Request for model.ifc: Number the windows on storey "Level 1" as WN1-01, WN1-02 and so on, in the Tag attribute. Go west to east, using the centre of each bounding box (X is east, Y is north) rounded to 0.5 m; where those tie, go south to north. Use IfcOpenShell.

First a look at what the model holds.

```python
import ifcopenshell
import ifcopenshell.util.element
import ifcopenshell.util.placement

model = ifcopenshell.open("model.ifc")
print(model.schema)
storey = next(s for s in model.by_type("IfcBuildingStorey") if s.Name == "Level 1")
windows = [e for e in ifcopenshell.util.element.get_decomposition(storey) if e.is_a("IfcWindow")]
for e in sorted(windows, key=lambda e: e.id()):
    origin = ifcopenshell.util.placement.get_local_placement(e.ObjectPlacement)[:3, 3]
    print(e.id(), e.Tag, e.Name, origin.round(2) + 0.0, sep=" | ")
```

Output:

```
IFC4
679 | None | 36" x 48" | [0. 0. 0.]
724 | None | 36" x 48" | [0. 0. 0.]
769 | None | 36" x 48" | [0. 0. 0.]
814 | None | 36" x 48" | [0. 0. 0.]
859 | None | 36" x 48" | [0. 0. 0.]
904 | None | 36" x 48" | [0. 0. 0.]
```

```python
import ifcopenshell
import ifcopenshell.geom
import ifcopenshell.util.element
import ifcopenshell.util.shape

model = ifcopenshell.open("model.ifc")
settings = ifcopenshell.geom.settings()
settings.set("use-world-coords", True)


def centre(element):
    shape = ifcopenshell.geom.create_shape(settings, element)
    return ifcopenshell.util.shape.get_bbox_centroid(shape.geometry)


storey = next(s for s in model.by_type("IfcBuildingStorey") if s.Name == "Level 1")
windows = [e for e in ifcopenshell.util.element.get_decomposition(storey) if e.is_a("IfcWindow")]

# Insertion points can sit at a corner or the storey origin, so sort by the geometry (in metres).
centres = {e: centre(e) for e in windows}
windows.sort(key=lambda e: (round(centres[e][0] / 0.5), centres[e][1]))

for i, e in enumerate(windows, start=1):
    number = f"WN1-{i:02d}"
    e.Tag = number
    print(e.id(), number)

model.write("model_v2.ifc")
```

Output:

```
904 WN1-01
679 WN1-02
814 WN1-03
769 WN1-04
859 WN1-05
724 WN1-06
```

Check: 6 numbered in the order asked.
